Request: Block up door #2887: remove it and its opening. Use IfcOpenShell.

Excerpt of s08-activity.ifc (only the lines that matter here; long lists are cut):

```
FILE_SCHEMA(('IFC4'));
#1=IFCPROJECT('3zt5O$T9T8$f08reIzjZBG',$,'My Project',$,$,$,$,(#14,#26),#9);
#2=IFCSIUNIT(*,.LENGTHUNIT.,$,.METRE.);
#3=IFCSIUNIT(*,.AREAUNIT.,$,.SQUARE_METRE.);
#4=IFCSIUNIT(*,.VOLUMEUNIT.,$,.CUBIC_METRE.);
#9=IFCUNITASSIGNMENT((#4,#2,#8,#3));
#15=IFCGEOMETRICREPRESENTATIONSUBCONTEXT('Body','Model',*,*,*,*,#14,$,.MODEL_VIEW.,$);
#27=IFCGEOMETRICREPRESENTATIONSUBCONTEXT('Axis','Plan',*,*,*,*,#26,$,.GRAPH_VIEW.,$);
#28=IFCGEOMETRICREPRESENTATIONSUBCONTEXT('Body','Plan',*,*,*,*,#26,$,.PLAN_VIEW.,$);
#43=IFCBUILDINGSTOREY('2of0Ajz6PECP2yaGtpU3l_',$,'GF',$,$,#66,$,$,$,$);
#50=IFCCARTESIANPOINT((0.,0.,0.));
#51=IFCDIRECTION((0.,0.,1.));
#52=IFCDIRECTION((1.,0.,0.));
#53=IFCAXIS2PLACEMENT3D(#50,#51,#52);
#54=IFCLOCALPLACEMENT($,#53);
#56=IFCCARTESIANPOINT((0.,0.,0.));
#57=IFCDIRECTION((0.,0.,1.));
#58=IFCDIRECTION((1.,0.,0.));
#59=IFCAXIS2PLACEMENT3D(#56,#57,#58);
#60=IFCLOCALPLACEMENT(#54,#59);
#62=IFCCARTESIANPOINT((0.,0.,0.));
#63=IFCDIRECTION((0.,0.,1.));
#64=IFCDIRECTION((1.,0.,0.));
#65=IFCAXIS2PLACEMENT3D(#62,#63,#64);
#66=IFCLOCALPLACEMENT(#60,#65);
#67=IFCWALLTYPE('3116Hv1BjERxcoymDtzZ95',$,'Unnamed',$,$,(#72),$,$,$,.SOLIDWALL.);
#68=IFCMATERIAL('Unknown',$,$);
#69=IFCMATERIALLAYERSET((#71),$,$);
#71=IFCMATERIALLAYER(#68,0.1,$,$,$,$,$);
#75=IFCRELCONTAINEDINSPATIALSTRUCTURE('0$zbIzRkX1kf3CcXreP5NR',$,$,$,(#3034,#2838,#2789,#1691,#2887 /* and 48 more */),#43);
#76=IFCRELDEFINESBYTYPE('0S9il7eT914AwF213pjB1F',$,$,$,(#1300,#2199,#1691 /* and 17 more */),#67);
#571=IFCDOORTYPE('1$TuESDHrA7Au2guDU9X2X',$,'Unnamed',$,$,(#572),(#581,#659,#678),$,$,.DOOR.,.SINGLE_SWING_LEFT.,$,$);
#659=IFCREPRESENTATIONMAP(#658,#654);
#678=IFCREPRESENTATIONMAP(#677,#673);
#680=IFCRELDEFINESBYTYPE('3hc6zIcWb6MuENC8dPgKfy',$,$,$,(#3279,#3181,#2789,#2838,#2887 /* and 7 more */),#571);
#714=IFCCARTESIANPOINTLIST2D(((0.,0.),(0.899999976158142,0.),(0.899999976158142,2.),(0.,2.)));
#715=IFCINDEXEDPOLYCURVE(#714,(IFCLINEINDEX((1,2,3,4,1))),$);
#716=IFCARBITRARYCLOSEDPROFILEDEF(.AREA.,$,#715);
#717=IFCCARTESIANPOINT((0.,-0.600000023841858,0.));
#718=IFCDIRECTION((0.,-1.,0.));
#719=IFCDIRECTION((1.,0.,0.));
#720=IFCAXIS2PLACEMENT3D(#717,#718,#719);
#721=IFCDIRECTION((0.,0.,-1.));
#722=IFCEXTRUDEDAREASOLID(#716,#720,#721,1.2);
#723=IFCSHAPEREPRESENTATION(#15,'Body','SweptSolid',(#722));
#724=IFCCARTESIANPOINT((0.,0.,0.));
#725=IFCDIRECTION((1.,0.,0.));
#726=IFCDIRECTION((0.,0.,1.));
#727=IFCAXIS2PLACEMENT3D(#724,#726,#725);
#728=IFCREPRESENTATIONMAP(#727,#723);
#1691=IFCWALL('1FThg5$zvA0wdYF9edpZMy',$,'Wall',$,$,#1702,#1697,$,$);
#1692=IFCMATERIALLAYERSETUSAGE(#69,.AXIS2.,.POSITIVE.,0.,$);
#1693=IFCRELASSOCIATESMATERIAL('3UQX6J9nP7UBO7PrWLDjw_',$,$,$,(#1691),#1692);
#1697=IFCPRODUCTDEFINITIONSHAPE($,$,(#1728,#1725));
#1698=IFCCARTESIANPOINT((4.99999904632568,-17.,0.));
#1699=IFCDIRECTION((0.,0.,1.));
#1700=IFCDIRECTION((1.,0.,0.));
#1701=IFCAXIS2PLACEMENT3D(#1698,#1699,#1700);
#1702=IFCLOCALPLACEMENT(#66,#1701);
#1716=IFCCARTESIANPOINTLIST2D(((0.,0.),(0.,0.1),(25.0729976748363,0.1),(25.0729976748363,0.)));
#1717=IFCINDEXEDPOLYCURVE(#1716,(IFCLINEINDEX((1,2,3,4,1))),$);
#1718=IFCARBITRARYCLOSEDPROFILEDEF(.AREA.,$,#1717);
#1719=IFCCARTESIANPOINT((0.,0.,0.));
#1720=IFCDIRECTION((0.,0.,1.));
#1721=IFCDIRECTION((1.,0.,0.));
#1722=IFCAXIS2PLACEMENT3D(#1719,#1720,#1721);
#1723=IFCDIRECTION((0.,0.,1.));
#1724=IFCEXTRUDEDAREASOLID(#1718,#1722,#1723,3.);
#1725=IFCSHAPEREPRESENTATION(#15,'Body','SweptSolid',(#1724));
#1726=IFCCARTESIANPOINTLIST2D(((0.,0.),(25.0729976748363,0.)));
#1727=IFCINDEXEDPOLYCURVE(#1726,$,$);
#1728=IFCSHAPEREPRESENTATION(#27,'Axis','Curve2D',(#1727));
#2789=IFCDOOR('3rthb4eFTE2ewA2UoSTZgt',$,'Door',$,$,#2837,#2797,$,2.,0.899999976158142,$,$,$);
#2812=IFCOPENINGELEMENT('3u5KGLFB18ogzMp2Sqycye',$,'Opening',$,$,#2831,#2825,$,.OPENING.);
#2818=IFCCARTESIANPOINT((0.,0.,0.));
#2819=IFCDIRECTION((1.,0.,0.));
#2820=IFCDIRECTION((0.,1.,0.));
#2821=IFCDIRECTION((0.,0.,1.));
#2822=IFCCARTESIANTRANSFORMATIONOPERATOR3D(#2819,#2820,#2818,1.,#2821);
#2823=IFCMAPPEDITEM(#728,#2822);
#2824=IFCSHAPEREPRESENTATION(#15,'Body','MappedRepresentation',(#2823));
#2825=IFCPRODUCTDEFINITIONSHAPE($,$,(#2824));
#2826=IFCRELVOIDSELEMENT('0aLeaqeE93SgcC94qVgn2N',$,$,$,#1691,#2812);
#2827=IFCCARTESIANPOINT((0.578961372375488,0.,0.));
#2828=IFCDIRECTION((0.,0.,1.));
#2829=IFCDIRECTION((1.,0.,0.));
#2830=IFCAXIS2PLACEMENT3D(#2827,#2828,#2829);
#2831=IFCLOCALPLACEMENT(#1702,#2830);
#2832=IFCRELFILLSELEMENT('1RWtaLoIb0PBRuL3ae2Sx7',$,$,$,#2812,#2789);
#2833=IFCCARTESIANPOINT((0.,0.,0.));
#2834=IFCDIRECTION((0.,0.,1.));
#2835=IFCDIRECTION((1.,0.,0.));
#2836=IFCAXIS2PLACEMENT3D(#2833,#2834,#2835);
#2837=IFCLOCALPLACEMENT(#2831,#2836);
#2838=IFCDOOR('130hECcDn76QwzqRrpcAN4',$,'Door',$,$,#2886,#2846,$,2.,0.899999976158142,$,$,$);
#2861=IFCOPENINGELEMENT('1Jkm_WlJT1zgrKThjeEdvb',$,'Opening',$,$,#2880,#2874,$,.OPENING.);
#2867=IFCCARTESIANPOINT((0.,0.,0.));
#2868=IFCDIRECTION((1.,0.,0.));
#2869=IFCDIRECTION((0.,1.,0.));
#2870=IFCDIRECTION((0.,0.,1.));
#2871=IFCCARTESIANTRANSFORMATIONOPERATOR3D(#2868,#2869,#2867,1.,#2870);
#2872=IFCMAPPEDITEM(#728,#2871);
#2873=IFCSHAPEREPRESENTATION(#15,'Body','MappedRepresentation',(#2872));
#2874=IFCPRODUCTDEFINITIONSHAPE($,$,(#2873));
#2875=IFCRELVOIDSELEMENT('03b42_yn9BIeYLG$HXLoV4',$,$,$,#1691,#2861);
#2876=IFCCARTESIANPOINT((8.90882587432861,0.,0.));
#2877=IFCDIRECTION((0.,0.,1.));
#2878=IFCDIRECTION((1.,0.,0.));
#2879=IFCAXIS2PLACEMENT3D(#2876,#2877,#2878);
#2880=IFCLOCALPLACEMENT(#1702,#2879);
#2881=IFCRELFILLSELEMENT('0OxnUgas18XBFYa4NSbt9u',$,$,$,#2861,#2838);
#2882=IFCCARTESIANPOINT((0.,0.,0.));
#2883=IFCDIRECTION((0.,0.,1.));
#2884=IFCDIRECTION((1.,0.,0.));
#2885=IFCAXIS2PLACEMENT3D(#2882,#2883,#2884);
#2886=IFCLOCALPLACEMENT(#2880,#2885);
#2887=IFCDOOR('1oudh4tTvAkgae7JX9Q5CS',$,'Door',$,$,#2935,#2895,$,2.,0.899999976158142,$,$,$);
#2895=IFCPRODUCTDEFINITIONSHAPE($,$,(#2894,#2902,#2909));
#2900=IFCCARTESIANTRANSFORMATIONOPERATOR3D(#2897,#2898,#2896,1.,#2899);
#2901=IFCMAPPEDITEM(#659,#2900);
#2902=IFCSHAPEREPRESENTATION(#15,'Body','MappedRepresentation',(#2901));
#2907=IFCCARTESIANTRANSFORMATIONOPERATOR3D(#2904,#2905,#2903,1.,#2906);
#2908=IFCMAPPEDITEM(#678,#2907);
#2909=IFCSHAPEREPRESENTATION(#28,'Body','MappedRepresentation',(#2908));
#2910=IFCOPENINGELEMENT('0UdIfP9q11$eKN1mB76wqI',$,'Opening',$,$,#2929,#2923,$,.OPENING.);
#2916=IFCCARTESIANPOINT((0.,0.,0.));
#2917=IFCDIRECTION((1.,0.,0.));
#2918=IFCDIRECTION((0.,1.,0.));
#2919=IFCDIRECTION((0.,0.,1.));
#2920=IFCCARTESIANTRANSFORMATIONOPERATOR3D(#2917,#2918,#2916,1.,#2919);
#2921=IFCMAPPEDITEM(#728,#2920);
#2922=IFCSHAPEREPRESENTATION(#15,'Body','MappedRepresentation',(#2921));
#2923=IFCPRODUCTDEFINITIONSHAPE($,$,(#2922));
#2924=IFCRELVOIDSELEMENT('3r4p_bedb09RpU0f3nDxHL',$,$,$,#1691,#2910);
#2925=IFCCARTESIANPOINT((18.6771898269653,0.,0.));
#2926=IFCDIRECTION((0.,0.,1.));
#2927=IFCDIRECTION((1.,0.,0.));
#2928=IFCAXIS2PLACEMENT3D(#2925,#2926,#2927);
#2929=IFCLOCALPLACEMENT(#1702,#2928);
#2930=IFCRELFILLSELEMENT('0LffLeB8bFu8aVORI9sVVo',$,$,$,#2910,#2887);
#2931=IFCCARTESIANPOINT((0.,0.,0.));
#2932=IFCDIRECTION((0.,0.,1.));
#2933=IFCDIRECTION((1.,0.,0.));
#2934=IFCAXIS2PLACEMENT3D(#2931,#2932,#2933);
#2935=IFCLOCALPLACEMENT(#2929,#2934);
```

```python
import ifcopenshell
import ifcopenshell.api.feature
import ifcopenshell.api.root
import ifcopenshell.geom
import ifcopenshell.util.shape

model = ifcopenshell.open("s08-activity.ifc")
settings = ifcopenshell.geom.settings()


def volume(element):
    """Net volume in cubic metres, openings subtracted."""
    shape = ifcopenshell.geom.create_shape(settings, element)
    return ifcopenshell.util.shape.get_volume(shape.geometry)


door = model.by_guid("1oudh4tTvAkgae7JX9Q5CS")
opening = door.FillsVoids[0].RelatingOpeningElement
wall = opening.VoidsElements[0].RelatingBuildingElement
before = volume(wall)

ifcopenshell.api.root.remove_product(model, product=door)
ifcopenshell.api.feature.remove_feature(model, feature=opening)

after = volume(wall)

print(f"wall volume {before:.3f} -> {after:.3f} m3")

model.write("s08-activity-out.ifc")
```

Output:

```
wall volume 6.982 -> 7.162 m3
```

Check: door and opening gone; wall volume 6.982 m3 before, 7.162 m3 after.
